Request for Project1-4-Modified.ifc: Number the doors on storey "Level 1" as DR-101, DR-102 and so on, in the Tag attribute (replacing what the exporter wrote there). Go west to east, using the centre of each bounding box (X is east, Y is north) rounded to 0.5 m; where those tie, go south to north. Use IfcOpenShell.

First a look at what the model holds.

```python
import ifcopenshell
import ifcopenshell.util.element
import ifcopenshell.util.placement

model = ifcopenshell.open("Project1-4-Modified.ifc")
print(model.schema)
storey = next(s for s in model.by_type("IfcBuildingStorey") if s.Name == "Level 1")
doors = [e for e in ifcopenshell.util.element.get_decomposition(storey) if e.is_a("IfcDoor")]
for e in sorted(doors, key=lambda e: e.id()):
    origin = ifcopenshell.util.placement.get_local_placement(e.ObjectPlacement)[:3, 3]
    print(e.id(), e.Tag, e.Name, origin.round(2) + 0.0, sep=" | ")
```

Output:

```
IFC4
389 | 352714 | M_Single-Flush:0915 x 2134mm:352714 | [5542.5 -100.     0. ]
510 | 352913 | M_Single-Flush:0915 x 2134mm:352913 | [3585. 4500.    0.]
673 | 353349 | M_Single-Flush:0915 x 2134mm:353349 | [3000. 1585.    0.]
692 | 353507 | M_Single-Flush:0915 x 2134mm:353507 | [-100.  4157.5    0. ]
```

```python
import ifcopenshell
import ifcopenshell.geom
import ifcopenshell.util.element
import ifcopenshell.util.shape

model = ifcopenshell.open("Project1-4-Modified.ifc")
settings = ifcopenshell.geom.settings()
settings.set("use-world-coords", True)


def centre(element):
    shape = ifcopenshell.geom.create_shape(settings, element)
    return ifcopenshell.util.shape.get_bbox_centroid(shape.geometry)


storey = next(s for s in model.by_type("IfcBuildingStorey") if s.Name == "Level 1")
doors = [e for e in ifcopenshell.util.element.get_decomposition(storey) if e.is_a("IfcDoor")]

# Insertion points can sit at a corner or the storey origin, so sort by the geometry (in metres).
centres = {e: centre(e) for e in doors}
doors.sort(key=lambda e: (round(centres[e][0] / 0.5), centres[e][1]))

for i, e in enumerate(doors, start=1):
    number = f"DR-1{i:02d}"
    e.Tag = number
    print(e.id(), number)

model.write("Project1-4-Modified_rev.ifc")
```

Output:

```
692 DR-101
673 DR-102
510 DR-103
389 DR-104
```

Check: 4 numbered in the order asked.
